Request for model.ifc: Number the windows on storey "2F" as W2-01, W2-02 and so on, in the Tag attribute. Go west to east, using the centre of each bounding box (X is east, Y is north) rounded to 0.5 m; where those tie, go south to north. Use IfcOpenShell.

First a look at what the model holds.

```python
import ifcopenshell
import ifcopenshell.util.element
import ifcopenshell.util.placement

model = ifcopenshell.open("model.ifc")
print(model.schema)
storey = next(s for s in model.by_type("IfcBuildingStorey") if s.Name == "2F")
windows = [e for e in ifcopenshell.util.element.get_decomposition(storey) if e.is_a("IfcWindow")]
for e in sorted(windows, key=lambda e: e.id()):
    origin = ifcopenshell.util.placement.get_local_placement(e.ObjectPlacement)[:3, 3]
    print(e.id(), e.Tag, e.Name, origin.round(2) + 0.0, sep=" | ")
```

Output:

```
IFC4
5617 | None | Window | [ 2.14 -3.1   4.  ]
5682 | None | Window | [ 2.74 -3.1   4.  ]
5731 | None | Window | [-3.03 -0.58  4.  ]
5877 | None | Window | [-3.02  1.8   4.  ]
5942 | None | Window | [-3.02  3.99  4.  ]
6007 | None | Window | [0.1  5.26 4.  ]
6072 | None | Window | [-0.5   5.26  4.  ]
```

```python
import ifcopenshell
import ifcopenshell.geom
import ifcopenshell.util.element
import ifcopenshell.util.shape

model = ifcopenshell.open("model.ifc")
settings = ifcopenshell.geom.settings()
settings.set("use-world-coords", True)


def centre(element):
    shape = ifcopenshell.geom.create_shape(settings, element)
    return ifcopenshell.util.shape.get_bbox_centroid(shape.geometry)


storey = next(s for s in model.by_type("IfcBuildingStorey") if s.Name == "2F")
windows = [e for e in ifcopenshell.util.element.get_decomposition(storey) if e.is_a("IfcWindow")]

# Insertion points can sit at a corner or the storey origin, so sort by the geometry (in metres).
centres = {e: centre(e) for e in windows}
windows.sort(key=lambda e: (round(centres[e][0] / 0.5), centres[e][1]))

for i, e in enumerate(windows, start=1):
    number = f"W2-{i:02d}"
    e.Tag = number
    print(e.id(), number)

model.write("model-out.ifc")
```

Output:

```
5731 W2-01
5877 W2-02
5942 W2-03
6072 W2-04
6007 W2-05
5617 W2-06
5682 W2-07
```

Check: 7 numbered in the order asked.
